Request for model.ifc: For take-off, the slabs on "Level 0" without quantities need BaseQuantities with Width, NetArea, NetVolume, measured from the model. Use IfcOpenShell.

First a look at what the model holds.

```python
import ifcopenshell
import ifcopenshell.util.element
import ifcopenshell.util.unit

model = ifcopenshell.open("model.ifc")
print(model.schema)
for unit_type in ("LENGTHUNIT", "AREAUNIT", "VOLUMEUNIT"):
    print(unit_type, ifcopenshell.util.unit.calculate_unit_scale(model, unit_type))
storey = next(s for s in model.by_type("IfcBuildingStorey") if s.Name == "Level 0")
slabs = [e for e in ifcopenshell.util.element.get_decomposition(storey) if e.is_a("IfcSlab")]
for e in sorted(slabs, key=lambda e: e.id()):
    print(e.id(), e.is_a(), e.Name, list(ifcopenshell.util.element.get_psets(e, qtos_only=True)), sep=" | ")
```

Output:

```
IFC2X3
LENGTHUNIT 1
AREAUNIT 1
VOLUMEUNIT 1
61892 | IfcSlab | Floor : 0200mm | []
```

```python
import ifcopenshell
import ifcopenshell.api.pset
import ifcopenshell.geom
import ifcopenshell.util.element
import ifcopenshell.util.shape
import ifcopenshell.util.unit

model = ifcopenshell.open("model.ifc")
unit_scale = ifcopenshell.util.unit.calculate_unit_scale(model)
area_scale = ifcopenshell.util.unit.calculate_unit_scale(model, "AREAUNIT")
volume_scale = ifcopenshell.util.unit.calculate_unit_scale(model, "VOLUMEUNIT")
settings = ifcopenshell.geom.settings()

storey = next(s for s in model.by_type("IfcBuildingStorey") if s.Name == "Level 0")
slabs = [e for e in ifcopenshell.util.element.get_decomposition(storey) if e.is_a("IfcSlab")]

for e in sorted(slabs, key=lambda e: e.id()):
    if ifcopenshell.util.element.get_psets(e, qtos_only=True, should_inherit=False):
        continue
    # Geometry comes back in metres, in the element's own axes.
    shape = ifcopenshell.geom.create_shape(settings, e)
    values = {
        "Width": ifcopenshell.util.shape.get_z(shape.geometry) / unit_scale,
        "NetArea": ifcopenshell.util.shape.get_footprint_area(shape.geometry) / area_scale,
        "NetVolume": ifcopenshell.util.shape.get_volume(shape.geometry) / volume_scale,
    }
    qto = ifcopenshell.api.pset.add_qto(model, product=e, name="BaseQuantities")
    ifcopenshell.api.pset.edit_qto(model, qto=qto, properties=values)
    print(e.id(), {k: round(v, 3) for k, v in values.items()})

model.write("model_updated.ifc")
```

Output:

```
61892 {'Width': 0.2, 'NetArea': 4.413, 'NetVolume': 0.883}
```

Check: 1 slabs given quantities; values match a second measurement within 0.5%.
